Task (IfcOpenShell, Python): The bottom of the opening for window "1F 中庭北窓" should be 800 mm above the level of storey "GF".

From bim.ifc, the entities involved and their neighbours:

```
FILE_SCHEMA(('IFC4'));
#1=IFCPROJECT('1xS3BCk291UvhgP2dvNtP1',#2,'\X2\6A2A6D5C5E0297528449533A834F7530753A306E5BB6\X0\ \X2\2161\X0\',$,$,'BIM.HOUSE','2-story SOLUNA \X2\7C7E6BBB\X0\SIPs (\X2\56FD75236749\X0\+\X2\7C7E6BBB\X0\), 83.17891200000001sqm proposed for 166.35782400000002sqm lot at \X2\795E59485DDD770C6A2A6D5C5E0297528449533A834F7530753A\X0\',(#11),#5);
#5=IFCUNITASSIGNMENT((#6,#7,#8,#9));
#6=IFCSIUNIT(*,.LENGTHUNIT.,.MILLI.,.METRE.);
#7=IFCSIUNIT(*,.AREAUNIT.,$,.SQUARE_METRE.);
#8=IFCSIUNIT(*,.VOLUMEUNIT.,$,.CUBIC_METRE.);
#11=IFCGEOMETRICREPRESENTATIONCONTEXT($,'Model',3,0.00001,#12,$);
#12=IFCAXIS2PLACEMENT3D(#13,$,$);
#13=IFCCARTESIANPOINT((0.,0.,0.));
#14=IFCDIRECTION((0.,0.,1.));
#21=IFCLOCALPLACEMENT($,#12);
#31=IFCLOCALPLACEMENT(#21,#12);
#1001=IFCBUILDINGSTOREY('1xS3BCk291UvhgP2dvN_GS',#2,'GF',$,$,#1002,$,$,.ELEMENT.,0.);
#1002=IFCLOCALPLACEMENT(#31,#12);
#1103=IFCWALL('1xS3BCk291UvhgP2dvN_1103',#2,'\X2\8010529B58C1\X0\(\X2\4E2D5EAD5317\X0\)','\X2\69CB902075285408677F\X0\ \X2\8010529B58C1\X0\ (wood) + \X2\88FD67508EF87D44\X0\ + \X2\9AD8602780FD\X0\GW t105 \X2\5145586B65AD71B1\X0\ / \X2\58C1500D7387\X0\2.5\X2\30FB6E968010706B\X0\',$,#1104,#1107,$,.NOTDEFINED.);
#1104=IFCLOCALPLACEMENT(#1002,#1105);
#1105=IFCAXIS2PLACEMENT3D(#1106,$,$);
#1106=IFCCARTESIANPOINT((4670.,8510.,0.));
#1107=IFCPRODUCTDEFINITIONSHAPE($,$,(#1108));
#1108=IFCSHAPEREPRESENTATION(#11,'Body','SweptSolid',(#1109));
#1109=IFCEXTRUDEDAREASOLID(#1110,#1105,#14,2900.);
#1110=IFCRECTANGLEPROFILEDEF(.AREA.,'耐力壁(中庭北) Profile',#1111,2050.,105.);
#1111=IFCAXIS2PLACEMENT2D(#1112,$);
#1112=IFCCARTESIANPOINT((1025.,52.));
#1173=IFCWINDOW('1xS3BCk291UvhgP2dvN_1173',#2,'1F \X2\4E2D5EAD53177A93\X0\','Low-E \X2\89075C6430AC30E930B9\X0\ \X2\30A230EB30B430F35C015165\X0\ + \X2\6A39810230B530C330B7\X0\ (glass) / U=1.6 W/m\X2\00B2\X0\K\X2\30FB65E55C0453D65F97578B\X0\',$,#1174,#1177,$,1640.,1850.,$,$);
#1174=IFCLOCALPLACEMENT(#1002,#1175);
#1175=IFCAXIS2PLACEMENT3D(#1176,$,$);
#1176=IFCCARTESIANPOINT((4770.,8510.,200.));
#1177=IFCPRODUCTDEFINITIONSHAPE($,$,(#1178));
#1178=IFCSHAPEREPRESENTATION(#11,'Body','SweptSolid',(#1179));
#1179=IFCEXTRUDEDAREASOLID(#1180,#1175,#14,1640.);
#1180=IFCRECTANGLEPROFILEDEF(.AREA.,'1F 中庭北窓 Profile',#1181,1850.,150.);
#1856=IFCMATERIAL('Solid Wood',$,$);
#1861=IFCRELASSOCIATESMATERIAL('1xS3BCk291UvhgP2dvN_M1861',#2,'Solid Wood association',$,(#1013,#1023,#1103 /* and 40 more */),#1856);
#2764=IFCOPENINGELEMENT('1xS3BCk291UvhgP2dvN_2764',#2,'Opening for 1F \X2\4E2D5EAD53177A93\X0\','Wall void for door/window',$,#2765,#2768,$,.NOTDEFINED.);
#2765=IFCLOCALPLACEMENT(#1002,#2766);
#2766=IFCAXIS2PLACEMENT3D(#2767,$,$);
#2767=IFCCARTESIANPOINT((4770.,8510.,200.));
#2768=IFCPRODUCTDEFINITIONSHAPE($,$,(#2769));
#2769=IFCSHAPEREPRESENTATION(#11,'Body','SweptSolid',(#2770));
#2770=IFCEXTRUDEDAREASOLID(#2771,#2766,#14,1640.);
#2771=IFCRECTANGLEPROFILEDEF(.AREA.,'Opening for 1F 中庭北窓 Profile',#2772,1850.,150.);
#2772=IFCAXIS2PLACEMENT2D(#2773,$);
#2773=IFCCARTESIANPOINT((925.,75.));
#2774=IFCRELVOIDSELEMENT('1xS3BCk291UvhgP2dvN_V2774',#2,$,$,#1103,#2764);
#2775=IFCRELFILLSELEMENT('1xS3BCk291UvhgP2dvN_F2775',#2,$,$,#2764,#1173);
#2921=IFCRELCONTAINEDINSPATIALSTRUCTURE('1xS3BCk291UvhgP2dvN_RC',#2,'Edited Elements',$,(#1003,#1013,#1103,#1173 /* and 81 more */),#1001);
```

```python
import numpy as np
import ifcopenshell
import ifcopenshell.api.geometry
import ifcopenshell.geom
import ifcopenshell.util.element
import ifcopenshell.util.placement
import ifcopenshell.util.shape
import ifcopenshell.util.unit

model = ifcopenshell.open("bim.ifc")
unit_scale = ifcopenshell.util.unit.calculate_unit_scale(model)

window = model.by_guid("1xS3BCk291UvhgP2dvN_1173")
opening = window.FillsVoids[0].RelatingOpeningElement
storey = ifcopenshell.util.element.get_container(window, ifc_class="IfcBuildingStorey")
level = ifcopenshell.util.placement.get_local_placement(storey.ObjectPlacement)[2, 3]

# The opening's origin need not be at the sill, so measure its lowest point.
shape = ifcopenshell.geom.create_shape(ifcopenshell.geom.settings(), opening)
bottom = ifcopenshell.util.shape.get_shape_bottom_elevation(shape, shape.geometry) / unit_scale
dz = level + 0.8 / unit_scale - bottom

shift = np.array([0.0, 0.0, dz])
# The window is not placed relative to its opening, so move both.
for product in (opening, window):
    matrix = ifcopenshell.util.placement.get_local_placement(product.ObjectPlacement)
    matrix[:3, 3] += shift
    ifcopenshell.api.geometry.edit_object_placement(model, product=product, matrix=matrix, is_si=False)

print(f"moved by {dz * unit_scale:+.3f} m")

model.write("bim_rev.ifc")
```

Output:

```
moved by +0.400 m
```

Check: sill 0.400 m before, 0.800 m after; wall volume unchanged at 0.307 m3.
